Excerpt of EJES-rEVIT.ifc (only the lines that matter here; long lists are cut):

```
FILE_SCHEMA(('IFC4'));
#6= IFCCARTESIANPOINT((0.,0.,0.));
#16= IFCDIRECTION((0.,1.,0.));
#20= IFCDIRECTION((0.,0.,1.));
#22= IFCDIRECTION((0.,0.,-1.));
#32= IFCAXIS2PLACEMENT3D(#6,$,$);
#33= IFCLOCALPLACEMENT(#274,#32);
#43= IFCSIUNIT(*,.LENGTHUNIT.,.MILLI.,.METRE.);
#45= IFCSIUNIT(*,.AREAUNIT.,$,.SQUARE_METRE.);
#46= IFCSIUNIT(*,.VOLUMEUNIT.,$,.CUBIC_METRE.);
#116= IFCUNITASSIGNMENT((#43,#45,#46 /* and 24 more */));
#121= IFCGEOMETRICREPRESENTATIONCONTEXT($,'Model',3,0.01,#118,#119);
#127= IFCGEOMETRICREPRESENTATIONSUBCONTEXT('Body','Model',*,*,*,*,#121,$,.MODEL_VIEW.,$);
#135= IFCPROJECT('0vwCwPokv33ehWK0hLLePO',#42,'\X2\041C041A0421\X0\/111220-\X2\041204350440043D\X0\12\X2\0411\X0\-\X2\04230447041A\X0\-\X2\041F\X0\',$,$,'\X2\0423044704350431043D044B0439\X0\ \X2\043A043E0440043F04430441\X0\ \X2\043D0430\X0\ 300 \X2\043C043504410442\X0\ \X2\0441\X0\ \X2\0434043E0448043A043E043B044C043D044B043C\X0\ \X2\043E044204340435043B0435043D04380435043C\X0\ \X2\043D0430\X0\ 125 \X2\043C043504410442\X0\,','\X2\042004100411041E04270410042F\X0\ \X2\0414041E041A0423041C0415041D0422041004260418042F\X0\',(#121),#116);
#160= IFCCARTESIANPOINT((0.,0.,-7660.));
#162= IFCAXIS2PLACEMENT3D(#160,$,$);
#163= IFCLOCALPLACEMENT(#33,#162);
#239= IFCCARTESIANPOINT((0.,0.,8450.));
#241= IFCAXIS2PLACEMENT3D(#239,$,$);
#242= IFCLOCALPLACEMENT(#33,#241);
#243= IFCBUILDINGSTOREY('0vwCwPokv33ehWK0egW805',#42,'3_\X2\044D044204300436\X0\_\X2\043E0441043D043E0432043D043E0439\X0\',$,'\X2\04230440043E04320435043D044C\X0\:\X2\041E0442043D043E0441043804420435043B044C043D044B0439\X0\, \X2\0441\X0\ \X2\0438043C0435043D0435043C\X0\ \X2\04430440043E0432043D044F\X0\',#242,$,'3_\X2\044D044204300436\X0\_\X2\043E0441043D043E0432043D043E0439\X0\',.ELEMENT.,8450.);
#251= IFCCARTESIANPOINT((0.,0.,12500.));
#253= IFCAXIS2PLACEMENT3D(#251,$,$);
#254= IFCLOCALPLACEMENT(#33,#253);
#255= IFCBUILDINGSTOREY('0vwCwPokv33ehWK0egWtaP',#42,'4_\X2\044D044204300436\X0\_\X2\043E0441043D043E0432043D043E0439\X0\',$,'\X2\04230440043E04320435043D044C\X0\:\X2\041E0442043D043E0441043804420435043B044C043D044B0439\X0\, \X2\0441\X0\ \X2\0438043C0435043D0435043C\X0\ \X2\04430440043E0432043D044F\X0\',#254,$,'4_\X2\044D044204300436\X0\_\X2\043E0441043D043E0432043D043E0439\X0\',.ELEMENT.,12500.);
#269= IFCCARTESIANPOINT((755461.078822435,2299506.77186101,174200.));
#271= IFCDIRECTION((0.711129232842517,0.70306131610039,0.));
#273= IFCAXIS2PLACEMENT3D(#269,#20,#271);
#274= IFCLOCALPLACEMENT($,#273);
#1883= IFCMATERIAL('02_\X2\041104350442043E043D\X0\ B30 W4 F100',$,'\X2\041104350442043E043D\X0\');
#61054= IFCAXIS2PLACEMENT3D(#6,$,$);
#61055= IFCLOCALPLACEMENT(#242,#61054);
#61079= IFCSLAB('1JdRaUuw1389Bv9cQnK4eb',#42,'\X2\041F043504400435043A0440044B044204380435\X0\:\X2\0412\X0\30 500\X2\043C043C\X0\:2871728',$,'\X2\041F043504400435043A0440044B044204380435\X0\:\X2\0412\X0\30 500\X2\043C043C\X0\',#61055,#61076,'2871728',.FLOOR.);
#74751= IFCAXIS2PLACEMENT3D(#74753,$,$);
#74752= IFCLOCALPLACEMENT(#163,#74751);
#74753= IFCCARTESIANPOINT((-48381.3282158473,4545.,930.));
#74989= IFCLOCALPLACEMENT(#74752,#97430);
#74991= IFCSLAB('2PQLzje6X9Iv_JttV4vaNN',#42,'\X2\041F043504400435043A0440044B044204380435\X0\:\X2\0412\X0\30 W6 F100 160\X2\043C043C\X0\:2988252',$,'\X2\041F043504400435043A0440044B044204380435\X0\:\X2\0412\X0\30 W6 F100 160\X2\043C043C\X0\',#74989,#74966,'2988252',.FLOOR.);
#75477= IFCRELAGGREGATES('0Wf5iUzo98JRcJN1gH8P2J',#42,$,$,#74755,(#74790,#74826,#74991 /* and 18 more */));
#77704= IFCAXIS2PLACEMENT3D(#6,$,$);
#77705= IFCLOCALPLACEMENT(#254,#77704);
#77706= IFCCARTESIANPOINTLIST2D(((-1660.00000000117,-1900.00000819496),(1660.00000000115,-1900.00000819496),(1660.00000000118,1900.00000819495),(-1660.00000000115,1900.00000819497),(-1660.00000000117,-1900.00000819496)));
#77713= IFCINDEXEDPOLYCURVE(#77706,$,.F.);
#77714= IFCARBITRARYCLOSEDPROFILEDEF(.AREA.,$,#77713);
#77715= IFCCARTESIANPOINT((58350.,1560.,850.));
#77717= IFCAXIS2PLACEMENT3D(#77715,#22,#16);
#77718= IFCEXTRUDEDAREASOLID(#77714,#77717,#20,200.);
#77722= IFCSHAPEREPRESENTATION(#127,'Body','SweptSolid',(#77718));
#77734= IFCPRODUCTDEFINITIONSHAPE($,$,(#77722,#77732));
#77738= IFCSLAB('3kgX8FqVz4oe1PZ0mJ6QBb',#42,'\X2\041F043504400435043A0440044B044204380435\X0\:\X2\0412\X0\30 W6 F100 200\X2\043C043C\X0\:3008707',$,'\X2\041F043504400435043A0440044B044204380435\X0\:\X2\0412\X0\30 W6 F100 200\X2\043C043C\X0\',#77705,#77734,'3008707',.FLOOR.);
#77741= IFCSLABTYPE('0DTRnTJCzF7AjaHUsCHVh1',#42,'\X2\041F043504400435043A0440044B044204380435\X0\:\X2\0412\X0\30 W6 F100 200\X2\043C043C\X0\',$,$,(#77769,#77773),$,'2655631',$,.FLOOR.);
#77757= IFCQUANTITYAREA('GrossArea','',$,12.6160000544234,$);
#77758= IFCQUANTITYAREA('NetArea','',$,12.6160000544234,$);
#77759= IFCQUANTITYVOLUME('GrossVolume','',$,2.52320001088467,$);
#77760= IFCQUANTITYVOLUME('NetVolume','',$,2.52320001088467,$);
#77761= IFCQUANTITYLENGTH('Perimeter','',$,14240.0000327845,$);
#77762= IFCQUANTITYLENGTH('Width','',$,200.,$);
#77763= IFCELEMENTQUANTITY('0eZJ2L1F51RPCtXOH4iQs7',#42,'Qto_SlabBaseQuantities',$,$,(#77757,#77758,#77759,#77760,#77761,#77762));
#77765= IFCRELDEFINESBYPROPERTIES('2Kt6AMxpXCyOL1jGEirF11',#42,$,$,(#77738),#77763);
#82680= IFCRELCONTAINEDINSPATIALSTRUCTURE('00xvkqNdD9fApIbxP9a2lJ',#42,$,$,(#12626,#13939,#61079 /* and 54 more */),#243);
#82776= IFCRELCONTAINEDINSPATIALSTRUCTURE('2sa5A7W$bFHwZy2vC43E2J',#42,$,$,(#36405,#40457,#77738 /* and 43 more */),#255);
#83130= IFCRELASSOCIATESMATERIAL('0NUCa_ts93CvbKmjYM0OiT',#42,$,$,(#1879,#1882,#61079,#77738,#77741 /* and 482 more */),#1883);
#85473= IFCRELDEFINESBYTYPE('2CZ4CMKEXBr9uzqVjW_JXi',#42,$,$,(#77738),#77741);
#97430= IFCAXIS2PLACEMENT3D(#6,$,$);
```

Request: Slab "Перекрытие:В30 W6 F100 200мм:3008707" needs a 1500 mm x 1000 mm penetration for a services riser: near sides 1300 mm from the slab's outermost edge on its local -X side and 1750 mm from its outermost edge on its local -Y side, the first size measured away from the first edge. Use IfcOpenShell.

```python
import numpy as np
import ifcopenshell
import ifcopenshell.api.feature
import ifcopenshell.api.geometry
import ifcopenshell.api.pset
import ifcopenshell.api.root
import ifcopenshell.geom
import ifcopenshell.util.element
import ifcopenshell.util.placement
import ifcopenshell.util.representation
import ifcopenshell.util.shape
import ifcopenshell.util.unit

model = ifcopenshell.open("EJES-rEVIT.ifc")
unit_scale = ifcopenshell.util.unit.calculate_unit_scale(model)
area_scale = ifcopenshell.util.unit.calculate_unit_scale(model, "AREAUNIT")
volume_scale = ifcopenshell.util.unit.calculate_unit_scale(model, "VOLUMEUNIT")
settings = ifcopenshell.geom.settings()


def volume(element):
    """Net volume in cubic metres, openings subtracted."""
    shape = ifcopenshell.geom.create_shape(settings, element)
    return ifcopenshell.util.shape.get_volume(shape.geometry)


slab = model.by_id(77738)
before = volume(slab)

# Extent in the slab's own axes, in metres. The edges named are its -X and -Y sides.
slab_shape = ifcopenshell.geom.create_shape(settings, slab)
vertices = ifcopenshell.util.shape.get_vertices(slab_shape.geometry)
x_min, y_min, bottom = vertices.min(axis=0)
top = vertices[:, 2].max()

opening = ifcopenshell.api.root.create_entity(model, ifc_class="IfcOpeningElement", name="Services riser opening", predefined_type="OPENING")
context = ifcopenshell.util.representation.get_context(model, "Model", "Body", "MODEL_VIEW")
width, depth = 1.5, 1
outline = [(0.0, 0.0), (width, 0.0), (width, depth), (0.0, depth), (0.0, 0.0)]
# Overshoot both faces by 50 mm so the cut is clean.
shape = ifcopenshell.api.geometry.add_slab_representation(
    model, context=context, depth=top - bottom + 0.1, polyline=outline
)
ifcopenshell.api.geometry.assign_representation(model, product=opening, representation=shape)

matrix = ifcopenshell.util.placement.get_local_placement(slab.ObjectPlacement)
matrix[:, 3] = matrix @ np.append(np.array([x_min + 1.3, y_min + 1.75, bottom - 0.05]) / unit_scale, 1.0)
ifcopenshell.api.geometry.edit_object_placement(model, product=opening, matrix=matrix, is_si=False)
ifcopenshell.api.feature.add_feature(model, feature=opening, element=slab)

after = volume(slab)

# Update the slab's stored quantities.
qto = model.by_id(ifcopenshell.util.element.get_pset(slab, "Qto_SlabBaseQuantities", should_inherit=False)["id"])
ifcopenshell.api.pset.edit_qto(model, qto=qto, properties={
    "NetArea": after / (top - bottom) / area_scale,
    "NetVolume": after / volume_scale,
})

print(f"slab volume {before:.3f} -> {after:.3f} m3")

model.write("EJES-rEVIT_v2.ifc")
```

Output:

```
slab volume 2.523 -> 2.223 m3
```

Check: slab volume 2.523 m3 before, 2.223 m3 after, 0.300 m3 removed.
